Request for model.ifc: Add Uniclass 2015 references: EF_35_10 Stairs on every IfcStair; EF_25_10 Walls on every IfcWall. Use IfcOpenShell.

First a look at what the model holds.

```python
import ifcopenshell

model = ifcopenshell.open("model.ifc")
print(model.schema)
print("classifications:", [c.Name for c in model.by_type("IfcClassification")])
for ifc_class in ("IfcDoor", "IfcRoof", "IfcStair", "IfcWall", "IfcWindow"):
    print(ifc_class, len(model.by_type(ifc_class)))
```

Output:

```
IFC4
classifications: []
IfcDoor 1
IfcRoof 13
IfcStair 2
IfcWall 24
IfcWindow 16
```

```python
import ifcopenshell
import ifcopenshell.api.classification

model = ifcopenshell.open("model.ifc")

system = ifcopenshell.api.classification.add_classification(model, classification="Uniclass 2015")

codes = {
    "IfcStair": ("EF_35_10", "Stairs"),
    "IfcWall": ("EF_25_10", "Walls"),
}
for ifc_class, (code, name) in codes.items():
    products = model.by_type(ifc_class)
    ifcopenshell.api.classification.add_reference(
        model, products=products, classification=system, identification=code, name=name
    )
    print(code, len(products))

model.write("model_edited.ifc")
```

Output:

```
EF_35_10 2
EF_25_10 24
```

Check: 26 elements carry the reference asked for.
